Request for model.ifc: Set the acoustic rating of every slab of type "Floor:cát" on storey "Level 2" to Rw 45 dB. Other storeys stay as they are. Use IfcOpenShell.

First a look at what the model holds.

```python
import ifcopenshell
import ifcopenshell.util.element

model = ifcopenshell.open("model.ifc")
print(model.schema)
storey = next(s for s in model.by_type("IfcBuildingStorey") if s.Name == "Level 2")
slabs = [e for e in ifcopenshell.util.element.get_decomposition(storey) if e.is_a("IfcSlab")]
seen = {}
for e in slabs:
    element_type = ifcopenshell.util.element.get_type(e)
    key = (element_type.Name if element_type != e and element_type else None, ifcopenshell.util.element.get_pset(e, "Pset_SlabCommon", "AcousticRating"))
    seen[key] = seen.get(key, 0) + 1
for (name, value), count in sorted(seen.items(), key=str):
    print(count, "x", name, "|", value)
```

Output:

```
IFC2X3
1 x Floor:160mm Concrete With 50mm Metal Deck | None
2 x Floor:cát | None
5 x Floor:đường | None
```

```python
import ifcopenshell
import ifcopenshell.api.pset
import ifcopenshell.util.element

model = ifcopenshell.open("model.ifc")

storey = next(s for s in model.by_type("IfcBuildingStorey") if s.Name == "Level 2")
slabs = [e for e in ifcopenshell.util.element.get_decomposition(storey) if e.is_a("IfcSlab")]

count = 0
for e in slabs:
    element_type = ifcopenshell.util.element.get_type(e)
    if element_type in (None, e) or element_type.Name != "Floor:cát":
        continue
    # add_pset returns the element's existing set when there is one.
    pset = ifcopenshell.api.pset.add_pset(model, product=e, name="Pset_SlabCommon")
    ifcopenshell.api.pset.edit_pset(model, pset=pset, properties={"AcousticRating": "Rw 45 dB"})
    count += 1

print(count, "slabs updated")

model.write("model-out.ifc")
```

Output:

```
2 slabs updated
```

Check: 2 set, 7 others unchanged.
